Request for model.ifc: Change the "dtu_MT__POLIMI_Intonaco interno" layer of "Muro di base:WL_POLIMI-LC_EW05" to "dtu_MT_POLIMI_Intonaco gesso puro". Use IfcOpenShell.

First a look at what the model holds.

```python
import ifcopenshell
import ifcopenshell.util.element

model = ifcopenshell.open("model.ifc")
print(model.schema)
for layer_set in model.by_type("IfcMaterialLayerSet"):
    if layer_set.LayerSetName == "Muro di base:WL_POLIMI-LC_EW05":
        for layer in layer_set.MaterialLayers:
            print(layer.id(), layer.Material and layer.Material.Name, layer.LayerThickness, sep=" | ")
        print(len(ifcopenshell.util.element.get_elements_by_material(model, layer_set)), "elements and types use it")
print(sorted(m.Name for m in model.by_type("IfcMaterial") if m.Name)[:60])
```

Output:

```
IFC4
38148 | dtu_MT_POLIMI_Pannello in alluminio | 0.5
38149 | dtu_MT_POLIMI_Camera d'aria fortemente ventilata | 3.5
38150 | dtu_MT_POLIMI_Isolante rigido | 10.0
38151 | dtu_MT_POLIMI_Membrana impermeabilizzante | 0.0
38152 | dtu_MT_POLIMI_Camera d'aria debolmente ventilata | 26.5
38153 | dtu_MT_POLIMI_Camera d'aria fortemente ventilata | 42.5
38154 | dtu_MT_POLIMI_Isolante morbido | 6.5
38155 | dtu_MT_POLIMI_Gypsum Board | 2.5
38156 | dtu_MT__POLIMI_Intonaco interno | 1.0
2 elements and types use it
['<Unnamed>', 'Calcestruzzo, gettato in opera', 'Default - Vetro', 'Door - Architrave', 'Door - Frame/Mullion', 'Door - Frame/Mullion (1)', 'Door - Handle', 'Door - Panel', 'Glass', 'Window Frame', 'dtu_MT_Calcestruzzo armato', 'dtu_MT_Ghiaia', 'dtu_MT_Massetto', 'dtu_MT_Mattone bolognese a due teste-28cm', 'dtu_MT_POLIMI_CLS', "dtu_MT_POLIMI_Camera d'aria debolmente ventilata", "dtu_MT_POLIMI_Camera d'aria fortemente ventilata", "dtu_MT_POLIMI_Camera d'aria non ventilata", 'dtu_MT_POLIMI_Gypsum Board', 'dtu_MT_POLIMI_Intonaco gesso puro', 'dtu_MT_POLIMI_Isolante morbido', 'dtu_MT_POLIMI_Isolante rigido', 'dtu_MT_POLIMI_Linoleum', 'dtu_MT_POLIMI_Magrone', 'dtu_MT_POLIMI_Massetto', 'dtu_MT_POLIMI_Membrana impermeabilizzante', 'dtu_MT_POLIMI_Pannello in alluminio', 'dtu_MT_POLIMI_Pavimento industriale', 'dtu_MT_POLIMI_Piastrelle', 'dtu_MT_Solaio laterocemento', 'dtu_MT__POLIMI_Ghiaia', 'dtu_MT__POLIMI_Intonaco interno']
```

```python
import ifcopenshell
import ifcopenshell.api.material

model = ifcopenshell.open("model.ifc")

layer_set = next(s for s in model.by_type("IfcMaterialLayerSet") if s.LayerSetName == "Muro di base:WL_POLIMI-LC_EW05")
layer = next(l for l in layer_set.MaterialLayers if l.Material and l.Material.Name == "dtu_MT__POLIMI_Intonaco interno")
material = next(m for m in model.by_type("IfcMaterial") if m.Name == "dtu_MT_POLIMI_Intonaco gesso puro")

# Point this one layer at the other material; renaming the old one would change it everywhere.
ifcopenshell.api.material.edit_layer(model, layer=layer, attributes={"Name": material.Name}, material=material)

print([l.Material.Name if l.Material else None for l in layer_set.MaterialLayers])

model.write("model-out.ifc")
```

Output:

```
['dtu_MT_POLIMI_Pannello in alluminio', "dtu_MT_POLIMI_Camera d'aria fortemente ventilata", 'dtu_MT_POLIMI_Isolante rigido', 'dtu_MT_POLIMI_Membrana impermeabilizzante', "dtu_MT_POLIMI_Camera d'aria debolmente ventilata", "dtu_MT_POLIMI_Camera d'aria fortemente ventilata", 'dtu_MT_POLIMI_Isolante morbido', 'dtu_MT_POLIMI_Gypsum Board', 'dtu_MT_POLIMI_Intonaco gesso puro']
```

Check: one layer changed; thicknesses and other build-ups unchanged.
